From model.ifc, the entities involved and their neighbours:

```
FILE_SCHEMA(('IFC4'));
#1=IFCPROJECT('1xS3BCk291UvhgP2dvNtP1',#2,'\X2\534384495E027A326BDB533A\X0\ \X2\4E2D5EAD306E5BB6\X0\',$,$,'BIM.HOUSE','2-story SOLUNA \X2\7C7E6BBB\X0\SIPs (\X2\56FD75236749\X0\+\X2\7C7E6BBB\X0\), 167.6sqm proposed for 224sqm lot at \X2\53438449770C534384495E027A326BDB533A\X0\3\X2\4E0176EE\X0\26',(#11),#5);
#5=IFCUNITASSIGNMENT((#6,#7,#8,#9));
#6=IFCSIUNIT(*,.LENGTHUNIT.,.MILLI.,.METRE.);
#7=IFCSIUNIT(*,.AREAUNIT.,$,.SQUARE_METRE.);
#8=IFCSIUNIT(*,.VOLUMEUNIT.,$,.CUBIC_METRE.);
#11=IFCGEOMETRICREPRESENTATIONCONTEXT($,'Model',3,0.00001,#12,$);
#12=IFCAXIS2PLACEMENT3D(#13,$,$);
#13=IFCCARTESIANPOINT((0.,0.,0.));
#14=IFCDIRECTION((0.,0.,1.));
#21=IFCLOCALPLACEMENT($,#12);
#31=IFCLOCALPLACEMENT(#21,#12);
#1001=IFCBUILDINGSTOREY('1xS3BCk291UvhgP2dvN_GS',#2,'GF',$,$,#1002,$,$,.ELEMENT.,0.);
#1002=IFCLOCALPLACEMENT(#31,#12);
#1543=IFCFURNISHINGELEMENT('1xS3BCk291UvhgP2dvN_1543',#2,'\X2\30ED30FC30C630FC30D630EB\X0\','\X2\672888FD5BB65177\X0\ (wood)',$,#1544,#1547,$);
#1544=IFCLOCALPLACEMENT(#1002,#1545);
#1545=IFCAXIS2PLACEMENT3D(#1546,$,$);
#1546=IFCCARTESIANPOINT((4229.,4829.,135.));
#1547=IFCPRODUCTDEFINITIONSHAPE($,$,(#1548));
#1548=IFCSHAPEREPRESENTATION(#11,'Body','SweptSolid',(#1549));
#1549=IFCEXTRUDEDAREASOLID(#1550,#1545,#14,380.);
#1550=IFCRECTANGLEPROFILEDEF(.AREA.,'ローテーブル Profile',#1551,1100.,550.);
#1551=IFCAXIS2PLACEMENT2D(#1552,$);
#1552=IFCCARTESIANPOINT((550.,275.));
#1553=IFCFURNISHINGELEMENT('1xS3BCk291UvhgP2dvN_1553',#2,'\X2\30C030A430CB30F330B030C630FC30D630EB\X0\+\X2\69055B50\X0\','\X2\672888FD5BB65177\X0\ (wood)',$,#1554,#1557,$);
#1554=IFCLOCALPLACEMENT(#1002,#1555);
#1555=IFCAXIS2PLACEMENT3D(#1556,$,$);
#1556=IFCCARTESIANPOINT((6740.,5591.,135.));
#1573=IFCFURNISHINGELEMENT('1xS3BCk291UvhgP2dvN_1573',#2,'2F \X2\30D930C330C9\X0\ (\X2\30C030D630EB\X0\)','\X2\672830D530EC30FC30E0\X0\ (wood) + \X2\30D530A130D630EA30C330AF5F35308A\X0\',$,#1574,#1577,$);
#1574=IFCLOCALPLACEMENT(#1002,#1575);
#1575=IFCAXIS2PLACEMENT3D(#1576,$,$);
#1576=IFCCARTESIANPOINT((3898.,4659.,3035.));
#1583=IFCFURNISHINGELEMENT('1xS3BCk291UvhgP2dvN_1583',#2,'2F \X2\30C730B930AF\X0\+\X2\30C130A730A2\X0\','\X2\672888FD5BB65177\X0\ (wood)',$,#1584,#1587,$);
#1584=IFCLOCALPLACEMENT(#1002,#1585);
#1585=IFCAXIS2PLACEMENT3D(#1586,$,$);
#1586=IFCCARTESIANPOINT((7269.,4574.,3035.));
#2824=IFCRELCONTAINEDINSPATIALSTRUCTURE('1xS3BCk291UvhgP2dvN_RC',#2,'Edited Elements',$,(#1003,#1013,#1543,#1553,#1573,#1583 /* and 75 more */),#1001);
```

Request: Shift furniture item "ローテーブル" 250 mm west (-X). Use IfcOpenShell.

```python
import ifcopenshell
import ifcopenshell.api.geometry
import ifcopenshell.util.placement

model = ifcopenshell.open("model.ifc")

item = model.by_guid("1xS3BCk291UvhgP2dvN_1543")
matrix = ifcopenshell.util.placement.get_local_placement(item.ObjectPlacement)
matrix[0, 3] -= 250.0
ifcopenshell.api.geometry.edit_object_placement(model, product=item, matrix=matrix, is_si=False)

print(ifcopenshell.util.placement.get_local_placement(item.ObjectPlacement).round(3) + 0.0)

model.write("model_rev.ifc")
```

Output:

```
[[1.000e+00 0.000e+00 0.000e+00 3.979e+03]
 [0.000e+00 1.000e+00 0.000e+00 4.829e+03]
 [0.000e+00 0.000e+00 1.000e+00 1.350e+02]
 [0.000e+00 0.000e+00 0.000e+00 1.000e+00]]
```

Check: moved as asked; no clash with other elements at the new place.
